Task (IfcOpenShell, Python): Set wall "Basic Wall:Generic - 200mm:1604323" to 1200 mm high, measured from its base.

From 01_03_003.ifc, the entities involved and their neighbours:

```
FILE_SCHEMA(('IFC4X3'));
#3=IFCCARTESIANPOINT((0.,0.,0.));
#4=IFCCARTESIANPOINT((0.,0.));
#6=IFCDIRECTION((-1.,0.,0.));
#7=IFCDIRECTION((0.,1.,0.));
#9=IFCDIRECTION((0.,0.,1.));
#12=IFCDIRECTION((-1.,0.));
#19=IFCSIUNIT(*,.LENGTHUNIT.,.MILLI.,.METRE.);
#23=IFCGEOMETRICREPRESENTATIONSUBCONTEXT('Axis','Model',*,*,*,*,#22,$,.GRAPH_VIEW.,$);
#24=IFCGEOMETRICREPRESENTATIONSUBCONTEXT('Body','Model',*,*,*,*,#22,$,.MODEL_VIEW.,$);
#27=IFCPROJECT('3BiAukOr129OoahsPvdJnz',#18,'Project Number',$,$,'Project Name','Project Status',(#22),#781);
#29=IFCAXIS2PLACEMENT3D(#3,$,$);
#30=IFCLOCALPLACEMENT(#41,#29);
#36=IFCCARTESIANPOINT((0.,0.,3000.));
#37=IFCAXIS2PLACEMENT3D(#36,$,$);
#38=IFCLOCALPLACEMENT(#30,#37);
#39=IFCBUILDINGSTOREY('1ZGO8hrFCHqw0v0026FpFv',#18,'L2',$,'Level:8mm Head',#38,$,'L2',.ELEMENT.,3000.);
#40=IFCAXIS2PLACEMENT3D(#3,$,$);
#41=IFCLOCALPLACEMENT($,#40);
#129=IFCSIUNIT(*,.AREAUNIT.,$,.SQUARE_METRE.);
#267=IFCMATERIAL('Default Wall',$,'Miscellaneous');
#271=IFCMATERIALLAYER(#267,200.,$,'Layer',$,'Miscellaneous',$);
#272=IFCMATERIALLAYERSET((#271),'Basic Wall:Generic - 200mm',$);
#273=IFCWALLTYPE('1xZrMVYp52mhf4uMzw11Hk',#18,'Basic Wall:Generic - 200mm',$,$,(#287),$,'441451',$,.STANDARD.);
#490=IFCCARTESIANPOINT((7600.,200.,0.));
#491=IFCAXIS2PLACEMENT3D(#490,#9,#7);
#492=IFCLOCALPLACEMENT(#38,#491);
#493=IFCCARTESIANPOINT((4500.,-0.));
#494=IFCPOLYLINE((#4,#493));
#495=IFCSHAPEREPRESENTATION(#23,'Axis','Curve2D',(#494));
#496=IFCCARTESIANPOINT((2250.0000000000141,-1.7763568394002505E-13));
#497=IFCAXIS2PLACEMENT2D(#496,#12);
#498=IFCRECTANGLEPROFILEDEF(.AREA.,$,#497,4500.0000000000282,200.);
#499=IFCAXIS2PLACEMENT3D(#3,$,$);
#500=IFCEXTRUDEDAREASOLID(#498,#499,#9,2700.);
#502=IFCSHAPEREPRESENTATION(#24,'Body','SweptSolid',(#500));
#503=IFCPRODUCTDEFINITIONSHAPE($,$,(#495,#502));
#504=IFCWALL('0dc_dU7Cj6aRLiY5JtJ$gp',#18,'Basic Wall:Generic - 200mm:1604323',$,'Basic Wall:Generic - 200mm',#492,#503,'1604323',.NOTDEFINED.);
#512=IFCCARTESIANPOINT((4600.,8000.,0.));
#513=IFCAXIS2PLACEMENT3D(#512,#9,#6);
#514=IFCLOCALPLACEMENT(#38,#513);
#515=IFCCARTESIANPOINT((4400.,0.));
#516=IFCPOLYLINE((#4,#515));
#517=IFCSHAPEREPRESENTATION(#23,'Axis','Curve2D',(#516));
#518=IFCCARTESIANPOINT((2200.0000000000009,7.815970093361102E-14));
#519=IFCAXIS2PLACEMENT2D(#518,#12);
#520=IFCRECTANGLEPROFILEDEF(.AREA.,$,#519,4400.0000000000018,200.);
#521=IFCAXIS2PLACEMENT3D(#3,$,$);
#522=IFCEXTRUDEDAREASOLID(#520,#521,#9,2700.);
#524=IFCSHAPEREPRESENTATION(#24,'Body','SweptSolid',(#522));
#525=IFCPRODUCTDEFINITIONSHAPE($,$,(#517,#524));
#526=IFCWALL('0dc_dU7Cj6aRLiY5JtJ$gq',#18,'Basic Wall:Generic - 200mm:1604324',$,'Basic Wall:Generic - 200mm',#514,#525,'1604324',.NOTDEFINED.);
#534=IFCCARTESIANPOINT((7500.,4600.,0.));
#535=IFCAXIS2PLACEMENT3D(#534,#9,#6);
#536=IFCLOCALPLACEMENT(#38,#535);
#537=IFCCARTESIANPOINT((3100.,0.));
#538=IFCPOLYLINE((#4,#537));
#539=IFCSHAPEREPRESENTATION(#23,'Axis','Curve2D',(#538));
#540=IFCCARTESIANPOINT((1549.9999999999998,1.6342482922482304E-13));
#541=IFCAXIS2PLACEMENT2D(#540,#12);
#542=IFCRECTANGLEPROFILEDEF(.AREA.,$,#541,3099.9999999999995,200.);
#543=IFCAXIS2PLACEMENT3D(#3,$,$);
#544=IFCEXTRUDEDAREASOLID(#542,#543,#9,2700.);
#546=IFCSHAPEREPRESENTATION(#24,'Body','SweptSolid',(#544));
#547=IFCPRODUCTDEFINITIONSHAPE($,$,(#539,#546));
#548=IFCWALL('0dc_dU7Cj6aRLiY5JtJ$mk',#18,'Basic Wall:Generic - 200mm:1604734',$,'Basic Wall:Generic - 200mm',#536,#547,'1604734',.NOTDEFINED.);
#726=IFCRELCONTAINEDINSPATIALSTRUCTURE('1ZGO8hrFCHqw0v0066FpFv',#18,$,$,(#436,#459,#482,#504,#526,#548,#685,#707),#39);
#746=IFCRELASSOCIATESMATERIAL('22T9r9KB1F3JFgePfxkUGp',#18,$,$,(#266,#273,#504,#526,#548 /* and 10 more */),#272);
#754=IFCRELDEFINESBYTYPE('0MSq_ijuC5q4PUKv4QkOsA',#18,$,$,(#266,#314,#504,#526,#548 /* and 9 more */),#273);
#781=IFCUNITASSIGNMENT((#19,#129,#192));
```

```python
import ifcopenshell
import ifcopenshell.geom
import ifcopenshell.util.representation
import ifcopenshell.util.shape
import ifcopenshell.util.unit

model = ifcopenshell.open("01_03_003.ifc")
unit_scale = ifcopenshell.util.unit.calculate_unit_scale(model)
settings = ifcopenshell.geom.settings()


def volume(element):
    """Net volume in cubic metres, openings subtracted."""
    shape = ifcopenshell.geom.create_shape(settings, element)
    return ifcopenshell.util.shape.get_volume(shape.geometry)


wall = model.by_id(504)
before = volume(wall)

body = ifcopenshell.util.representation.get_representation(wall, "Model", "Body")
solid = body.Items[0]
old_height = solid.Depth
solid.Depth = 1.2 / unit_scale
after = volume(wall)

print(f"height {old_height:g} -> {solid.Depth:g}, volume {before:.3f} -> {after:.3f} m3")

model.write("01_03_003_rev.ifc")
```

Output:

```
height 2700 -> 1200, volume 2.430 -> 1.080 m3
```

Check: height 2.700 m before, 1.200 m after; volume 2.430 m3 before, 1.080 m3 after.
